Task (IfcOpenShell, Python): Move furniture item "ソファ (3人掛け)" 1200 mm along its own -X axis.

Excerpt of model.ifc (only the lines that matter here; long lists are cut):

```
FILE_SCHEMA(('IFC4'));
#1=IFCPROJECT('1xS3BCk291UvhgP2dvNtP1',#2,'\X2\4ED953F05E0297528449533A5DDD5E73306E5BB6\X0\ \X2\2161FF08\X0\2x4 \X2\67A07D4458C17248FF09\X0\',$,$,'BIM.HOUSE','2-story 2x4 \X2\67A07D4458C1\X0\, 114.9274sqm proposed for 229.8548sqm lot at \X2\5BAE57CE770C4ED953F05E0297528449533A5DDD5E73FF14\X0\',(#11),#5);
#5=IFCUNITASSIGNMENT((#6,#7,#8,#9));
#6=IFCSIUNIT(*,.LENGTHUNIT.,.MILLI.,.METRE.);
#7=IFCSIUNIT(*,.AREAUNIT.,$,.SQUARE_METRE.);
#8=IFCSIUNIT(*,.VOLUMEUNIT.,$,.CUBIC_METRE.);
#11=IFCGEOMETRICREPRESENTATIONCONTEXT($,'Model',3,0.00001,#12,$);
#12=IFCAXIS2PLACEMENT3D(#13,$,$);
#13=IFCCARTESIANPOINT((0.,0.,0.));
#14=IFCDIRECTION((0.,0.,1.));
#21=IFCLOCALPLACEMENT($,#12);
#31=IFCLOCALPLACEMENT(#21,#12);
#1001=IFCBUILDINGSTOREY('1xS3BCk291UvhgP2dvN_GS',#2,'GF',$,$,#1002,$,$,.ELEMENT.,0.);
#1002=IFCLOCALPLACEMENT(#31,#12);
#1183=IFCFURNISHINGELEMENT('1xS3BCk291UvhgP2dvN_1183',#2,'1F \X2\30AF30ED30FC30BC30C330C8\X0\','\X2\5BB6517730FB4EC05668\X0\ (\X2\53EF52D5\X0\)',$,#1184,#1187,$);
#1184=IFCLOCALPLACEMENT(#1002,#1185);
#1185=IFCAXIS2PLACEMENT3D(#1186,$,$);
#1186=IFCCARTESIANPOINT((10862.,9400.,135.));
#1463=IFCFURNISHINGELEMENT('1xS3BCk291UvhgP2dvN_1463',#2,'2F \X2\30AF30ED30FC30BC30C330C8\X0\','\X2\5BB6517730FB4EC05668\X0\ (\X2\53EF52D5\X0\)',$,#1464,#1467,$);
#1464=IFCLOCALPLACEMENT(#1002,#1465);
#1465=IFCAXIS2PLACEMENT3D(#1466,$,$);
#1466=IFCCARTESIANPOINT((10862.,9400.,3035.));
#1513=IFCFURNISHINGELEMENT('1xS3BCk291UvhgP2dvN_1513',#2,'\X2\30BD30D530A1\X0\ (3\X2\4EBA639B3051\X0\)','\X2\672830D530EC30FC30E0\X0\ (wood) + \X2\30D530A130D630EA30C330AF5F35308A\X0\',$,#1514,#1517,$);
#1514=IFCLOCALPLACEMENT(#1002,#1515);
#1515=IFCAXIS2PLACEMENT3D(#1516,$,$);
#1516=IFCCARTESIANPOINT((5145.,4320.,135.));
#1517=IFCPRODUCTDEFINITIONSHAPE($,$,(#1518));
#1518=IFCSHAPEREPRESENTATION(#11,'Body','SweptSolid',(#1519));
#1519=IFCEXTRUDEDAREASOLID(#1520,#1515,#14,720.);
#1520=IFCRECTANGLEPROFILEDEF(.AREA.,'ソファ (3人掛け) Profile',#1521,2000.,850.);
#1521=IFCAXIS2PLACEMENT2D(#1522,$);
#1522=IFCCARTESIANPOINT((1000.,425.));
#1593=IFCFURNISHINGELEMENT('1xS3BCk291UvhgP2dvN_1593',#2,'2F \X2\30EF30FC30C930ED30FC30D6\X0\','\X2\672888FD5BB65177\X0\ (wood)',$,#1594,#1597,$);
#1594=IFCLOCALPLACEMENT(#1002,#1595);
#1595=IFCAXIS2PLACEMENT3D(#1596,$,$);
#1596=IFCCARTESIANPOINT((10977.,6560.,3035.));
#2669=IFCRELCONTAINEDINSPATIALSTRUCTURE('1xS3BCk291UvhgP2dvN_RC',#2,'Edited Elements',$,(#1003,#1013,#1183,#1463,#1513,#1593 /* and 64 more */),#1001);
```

```python
import ifcopenshell
import ifcopenshell.api.geometry
import ifcopenshell.util.placement
import ifcopenshell.util.unit

model = ifcopenshell.open("model.ifc")
unit_scale = ifcopenshell.util.unit.calculate_unit_scale(model)

item = model.by_guid("1xS3BCk291UvhgP2dvN_1513")
matrix = ifcopenshell.util.placement.get_local_placement(item.ObjectPlacement)
matrix[:3, 3] -= matrix[:3, 0] * 1.2 / unit_scale
ifcopenshell.api.geometry.edit_object_placement(model, product=item, matrix=matrix, is_si=False)

print(ifcopenshell.util.placement.get_local_placement(item.ObjectPlacement).round(3) + 0.0)

model.write("model_edited.ifc")
```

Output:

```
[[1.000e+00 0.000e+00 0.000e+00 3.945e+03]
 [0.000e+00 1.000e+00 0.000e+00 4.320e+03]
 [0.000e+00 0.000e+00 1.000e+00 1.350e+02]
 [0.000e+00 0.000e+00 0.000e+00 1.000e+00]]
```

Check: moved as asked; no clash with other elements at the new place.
